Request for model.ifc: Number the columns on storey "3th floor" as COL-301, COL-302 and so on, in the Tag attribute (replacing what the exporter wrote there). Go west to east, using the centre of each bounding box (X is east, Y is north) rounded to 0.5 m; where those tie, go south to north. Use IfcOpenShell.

First a look at what the model holds.

```python
import ifcopenshell
import ifcopenshell.util.element
import ifcopenshell.util.placement

model = ifcopenshell.open("model.ifc")
print(model.schema)
storey = next(s for s in model.by_type("IfcBuildingStorey") if s.Name == "3th floor")
columns = [e for e in ifcopenshell.util.element.get_decomposition(storey) if e.is_a("IfcColumn")]
for e in sorted(columns, key=lambda e: e.id()):
    origin = ifcopenshell.util.placement.get_local_placement(e.ObjectPlacement)[:3, 3]
    print(e.id(), e.Tag, e.Name, origin.round(2) + 0.0, sep=" | ")
```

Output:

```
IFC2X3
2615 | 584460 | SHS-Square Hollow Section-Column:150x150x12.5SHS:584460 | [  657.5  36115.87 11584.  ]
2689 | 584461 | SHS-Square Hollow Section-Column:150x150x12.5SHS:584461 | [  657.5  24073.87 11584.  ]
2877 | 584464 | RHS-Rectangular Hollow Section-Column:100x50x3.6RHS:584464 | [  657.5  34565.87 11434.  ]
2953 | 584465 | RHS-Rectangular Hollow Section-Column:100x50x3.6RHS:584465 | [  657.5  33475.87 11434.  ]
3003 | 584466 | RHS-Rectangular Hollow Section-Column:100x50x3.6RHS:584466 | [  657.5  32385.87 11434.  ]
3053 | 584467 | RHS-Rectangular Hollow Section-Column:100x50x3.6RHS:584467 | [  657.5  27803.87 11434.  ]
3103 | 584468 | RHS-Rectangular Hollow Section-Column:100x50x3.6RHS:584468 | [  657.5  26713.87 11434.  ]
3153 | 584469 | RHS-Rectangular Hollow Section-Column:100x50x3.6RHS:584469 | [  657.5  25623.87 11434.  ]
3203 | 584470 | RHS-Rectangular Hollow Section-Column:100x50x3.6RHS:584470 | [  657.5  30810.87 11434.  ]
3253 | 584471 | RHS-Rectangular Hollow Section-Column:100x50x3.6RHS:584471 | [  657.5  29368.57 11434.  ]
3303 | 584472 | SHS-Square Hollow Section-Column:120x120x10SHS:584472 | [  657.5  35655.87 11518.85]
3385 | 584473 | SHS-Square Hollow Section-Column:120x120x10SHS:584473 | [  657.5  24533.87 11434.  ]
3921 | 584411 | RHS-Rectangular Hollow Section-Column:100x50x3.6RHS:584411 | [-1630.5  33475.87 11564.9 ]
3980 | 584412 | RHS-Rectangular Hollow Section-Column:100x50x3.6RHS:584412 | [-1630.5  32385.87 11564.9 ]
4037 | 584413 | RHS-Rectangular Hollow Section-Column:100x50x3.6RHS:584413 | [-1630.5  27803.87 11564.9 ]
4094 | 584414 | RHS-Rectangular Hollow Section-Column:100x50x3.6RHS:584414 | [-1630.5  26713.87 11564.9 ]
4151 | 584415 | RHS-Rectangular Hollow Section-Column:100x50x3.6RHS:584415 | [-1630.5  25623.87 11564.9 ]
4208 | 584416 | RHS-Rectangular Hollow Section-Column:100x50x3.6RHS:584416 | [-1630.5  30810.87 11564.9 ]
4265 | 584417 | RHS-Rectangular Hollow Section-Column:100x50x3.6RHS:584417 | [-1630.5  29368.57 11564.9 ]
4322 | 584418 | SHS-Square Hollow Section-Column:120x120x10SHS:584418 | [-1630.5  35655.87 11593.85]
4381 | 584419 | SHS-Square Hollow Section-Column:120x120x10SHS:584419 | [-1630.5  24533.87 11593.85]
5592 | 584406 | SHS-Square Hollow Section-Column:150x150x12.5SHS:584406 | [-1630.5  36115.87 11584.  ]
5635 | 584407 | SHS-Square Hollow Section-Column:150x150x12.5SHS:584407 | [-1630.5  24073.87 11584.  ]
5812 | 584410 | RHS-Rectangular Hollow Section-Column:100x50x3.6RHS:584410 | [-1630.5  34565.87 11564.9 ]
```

```python
import ifcopenshell
import ifcopenshell.geom
import ifcopenshell.util.element
import ifcopenshell.util.shape

model = ifcopenshell.open("model.ifc")
settings = ifcopenshell.geom.settings()
settings.set("use-world-coords", True)


def centre(element):
    shape = ifcopenshell.geom.create_shape(settings, element)
    return ifcopenshell.util.shape.get_bbox_centroid(shape.geometry)


storey = next(s for s in model.by_type("IfcBuildingStorey") if s.Name == "3th floor")
columns = [e for e in ifcopenshell.util.element.get_decomposition(storey) if e.is_a("IfcColumn")]

# Insertion points can sit at a corner or the storey origin, so sort by the geometry (in metres).
centres = {e: centre(e) for e in columns}
columns.sort(key=lambda e: (round(centres[e][0] / 0.5), centres[e][1]))

for i, e in enumerate(columns, start=1):
    number = f"COL-3{i:02d}"
    e.Tag = number
    print(e.id(), number)

model.write("model_rev.ifc")
```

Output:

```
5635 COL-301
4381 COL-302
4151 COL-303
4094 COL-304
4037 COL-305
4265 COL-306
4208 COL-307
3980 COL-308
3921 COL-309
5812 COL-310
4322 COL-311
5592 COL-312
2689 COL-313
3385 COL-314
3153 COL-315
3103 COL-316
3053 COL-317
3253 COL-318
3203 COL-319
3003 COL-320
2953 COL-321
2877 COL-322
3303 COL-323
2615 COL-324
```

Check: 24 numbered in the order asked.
